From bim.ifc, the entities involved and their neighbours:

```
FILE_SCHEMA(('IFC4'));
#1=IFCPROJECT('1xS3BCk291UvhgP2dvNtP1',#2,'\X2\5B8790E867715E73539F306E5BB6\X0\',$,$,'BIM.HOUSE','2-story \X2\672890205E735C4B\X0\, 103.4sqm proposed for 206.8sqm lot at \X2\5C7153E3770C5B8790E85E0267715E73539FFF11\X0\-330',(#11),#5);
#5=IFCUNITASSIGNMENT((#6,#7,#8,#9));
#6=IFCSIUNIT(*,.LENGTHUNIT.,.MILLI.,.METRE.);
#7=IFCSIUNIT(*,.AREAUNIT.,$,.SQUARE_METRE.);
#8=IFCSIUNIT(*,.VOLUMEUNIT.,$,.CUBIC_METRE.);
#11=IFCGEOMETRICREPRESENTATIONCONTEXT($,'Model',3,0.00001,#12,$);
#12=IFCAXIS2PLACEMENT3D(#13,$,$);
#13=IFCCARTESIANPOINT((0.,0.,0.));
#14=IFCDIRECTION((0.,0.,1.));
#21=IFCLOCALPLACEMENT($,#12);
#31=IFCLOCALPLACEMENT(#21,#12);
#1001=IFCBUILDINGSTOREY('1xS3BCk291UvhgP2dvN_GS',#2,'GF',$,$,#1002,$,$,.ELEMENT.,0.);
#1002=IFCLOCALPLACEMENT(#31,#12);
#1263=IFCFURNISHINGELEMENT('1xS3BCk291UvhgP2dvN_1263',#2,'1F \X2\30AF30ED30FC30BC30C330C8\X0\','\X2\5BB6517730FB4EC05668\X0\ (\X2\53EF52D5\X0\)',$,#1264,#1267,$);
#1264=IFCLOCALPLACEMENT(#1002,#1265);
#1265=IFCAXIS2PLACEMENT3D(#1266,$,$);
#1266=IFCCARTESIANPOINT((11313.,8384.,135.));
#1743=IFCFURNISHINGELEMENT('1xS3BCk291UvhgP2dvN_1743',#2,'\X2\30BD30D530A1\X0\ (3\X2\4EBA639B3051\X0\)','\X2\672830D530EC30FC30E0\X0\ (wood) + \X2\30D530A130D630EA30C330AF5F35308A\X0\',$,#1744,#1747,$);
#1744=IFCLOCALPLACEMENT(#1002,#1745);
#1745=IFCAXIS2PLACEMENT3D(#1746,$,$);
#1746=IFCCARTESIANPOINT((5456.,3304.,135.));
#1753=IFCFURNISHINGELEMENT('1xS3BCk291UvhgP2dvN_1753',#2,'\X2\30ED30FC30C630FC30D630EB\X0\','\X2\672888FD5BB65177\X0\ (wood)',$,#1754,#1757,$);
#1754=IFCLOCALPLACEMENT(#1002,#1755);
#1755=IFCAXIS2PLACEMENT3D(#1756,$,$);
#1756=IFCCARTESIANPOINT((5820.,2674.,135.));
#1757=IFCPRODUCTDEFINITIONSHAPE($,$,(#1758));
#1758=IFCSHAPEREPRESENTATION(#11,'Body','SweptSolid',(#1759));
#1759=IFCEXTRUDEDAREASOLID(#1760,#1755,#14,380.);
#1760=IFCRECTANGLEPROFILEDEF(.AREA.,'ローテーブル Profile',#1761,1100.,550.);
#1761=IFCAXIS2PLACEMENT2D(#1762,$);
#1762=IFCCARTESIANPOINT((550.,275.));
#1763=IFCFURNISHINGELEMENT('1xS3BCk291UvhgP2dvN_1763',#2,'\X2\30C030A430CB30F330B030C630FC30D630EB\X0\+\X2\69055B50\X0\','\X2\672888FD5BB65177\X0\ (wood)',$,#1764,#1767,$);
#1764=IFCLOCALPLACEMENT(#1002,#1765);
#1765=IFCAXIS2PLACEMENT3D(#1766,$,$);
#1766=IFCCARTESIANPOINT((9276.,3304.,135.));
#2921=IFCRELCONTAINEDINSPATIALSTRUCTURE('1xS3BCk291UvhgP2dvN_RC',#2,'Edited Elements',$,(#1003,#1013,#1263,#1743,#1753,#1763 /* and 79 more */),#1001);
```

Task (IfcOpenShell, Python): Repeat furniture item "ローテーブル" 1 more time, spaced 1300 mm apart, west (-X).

```python
import numpy as np
import ifcopenshell
import ifcopenshell.api.geometry
import ifcopenshell.api.root
import ifcopenshell.util.element
import ifcopenshell.util.placement

model = ifcopenshell.open("bim.ifc")


def reuse_history(source, copy):
    """copy_class also copies each property set's owner history, people and application; keep the originals."""
    for rel in copy.IsDefinedBy:
        if rel.is_a("IfcRelDefinesByProperties") and (history := rel.RelatingPropertyDefinition.OwnerHistory):
            rel.RelatingPropertyDefinition.OwnerHistory = source.OwnerHistory
            ifcopenshell.util.element.remove_deep2(model, history)


source = model.by_guid("1xS3BCk291UvhgP2dvN_1753")
base = ifcopenshell.util.placement.get_local_placement(source.ObjectPlacement)
step = np.array([-1.0, 0.0, 0.0]) * 1300.0

for i in range(1, 2):
    copy = ifcopenshell.api.root.copy_class(model, product=source)
    copy.Representation = ifcopenshell.util.element.copy_deep(
        model, source.Representation, exclude=["IfcGeometricRepresentationContext", "IfcRepresentationMap"]
    )
    reuse_history(source, copy)
    matrix = base.copy()
    matrix[:3, 3] += i * step
    print("added at", matrix[:3, 3].round(3) + 0.0)
    ifcopenshell.api.geometry.edit_object_placement(model, product=copy, matrix=matrix, is_si=False)

model.write("bim_v2.ifc")
```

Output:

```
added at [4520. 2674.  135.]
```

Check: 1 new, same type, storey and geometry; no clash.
